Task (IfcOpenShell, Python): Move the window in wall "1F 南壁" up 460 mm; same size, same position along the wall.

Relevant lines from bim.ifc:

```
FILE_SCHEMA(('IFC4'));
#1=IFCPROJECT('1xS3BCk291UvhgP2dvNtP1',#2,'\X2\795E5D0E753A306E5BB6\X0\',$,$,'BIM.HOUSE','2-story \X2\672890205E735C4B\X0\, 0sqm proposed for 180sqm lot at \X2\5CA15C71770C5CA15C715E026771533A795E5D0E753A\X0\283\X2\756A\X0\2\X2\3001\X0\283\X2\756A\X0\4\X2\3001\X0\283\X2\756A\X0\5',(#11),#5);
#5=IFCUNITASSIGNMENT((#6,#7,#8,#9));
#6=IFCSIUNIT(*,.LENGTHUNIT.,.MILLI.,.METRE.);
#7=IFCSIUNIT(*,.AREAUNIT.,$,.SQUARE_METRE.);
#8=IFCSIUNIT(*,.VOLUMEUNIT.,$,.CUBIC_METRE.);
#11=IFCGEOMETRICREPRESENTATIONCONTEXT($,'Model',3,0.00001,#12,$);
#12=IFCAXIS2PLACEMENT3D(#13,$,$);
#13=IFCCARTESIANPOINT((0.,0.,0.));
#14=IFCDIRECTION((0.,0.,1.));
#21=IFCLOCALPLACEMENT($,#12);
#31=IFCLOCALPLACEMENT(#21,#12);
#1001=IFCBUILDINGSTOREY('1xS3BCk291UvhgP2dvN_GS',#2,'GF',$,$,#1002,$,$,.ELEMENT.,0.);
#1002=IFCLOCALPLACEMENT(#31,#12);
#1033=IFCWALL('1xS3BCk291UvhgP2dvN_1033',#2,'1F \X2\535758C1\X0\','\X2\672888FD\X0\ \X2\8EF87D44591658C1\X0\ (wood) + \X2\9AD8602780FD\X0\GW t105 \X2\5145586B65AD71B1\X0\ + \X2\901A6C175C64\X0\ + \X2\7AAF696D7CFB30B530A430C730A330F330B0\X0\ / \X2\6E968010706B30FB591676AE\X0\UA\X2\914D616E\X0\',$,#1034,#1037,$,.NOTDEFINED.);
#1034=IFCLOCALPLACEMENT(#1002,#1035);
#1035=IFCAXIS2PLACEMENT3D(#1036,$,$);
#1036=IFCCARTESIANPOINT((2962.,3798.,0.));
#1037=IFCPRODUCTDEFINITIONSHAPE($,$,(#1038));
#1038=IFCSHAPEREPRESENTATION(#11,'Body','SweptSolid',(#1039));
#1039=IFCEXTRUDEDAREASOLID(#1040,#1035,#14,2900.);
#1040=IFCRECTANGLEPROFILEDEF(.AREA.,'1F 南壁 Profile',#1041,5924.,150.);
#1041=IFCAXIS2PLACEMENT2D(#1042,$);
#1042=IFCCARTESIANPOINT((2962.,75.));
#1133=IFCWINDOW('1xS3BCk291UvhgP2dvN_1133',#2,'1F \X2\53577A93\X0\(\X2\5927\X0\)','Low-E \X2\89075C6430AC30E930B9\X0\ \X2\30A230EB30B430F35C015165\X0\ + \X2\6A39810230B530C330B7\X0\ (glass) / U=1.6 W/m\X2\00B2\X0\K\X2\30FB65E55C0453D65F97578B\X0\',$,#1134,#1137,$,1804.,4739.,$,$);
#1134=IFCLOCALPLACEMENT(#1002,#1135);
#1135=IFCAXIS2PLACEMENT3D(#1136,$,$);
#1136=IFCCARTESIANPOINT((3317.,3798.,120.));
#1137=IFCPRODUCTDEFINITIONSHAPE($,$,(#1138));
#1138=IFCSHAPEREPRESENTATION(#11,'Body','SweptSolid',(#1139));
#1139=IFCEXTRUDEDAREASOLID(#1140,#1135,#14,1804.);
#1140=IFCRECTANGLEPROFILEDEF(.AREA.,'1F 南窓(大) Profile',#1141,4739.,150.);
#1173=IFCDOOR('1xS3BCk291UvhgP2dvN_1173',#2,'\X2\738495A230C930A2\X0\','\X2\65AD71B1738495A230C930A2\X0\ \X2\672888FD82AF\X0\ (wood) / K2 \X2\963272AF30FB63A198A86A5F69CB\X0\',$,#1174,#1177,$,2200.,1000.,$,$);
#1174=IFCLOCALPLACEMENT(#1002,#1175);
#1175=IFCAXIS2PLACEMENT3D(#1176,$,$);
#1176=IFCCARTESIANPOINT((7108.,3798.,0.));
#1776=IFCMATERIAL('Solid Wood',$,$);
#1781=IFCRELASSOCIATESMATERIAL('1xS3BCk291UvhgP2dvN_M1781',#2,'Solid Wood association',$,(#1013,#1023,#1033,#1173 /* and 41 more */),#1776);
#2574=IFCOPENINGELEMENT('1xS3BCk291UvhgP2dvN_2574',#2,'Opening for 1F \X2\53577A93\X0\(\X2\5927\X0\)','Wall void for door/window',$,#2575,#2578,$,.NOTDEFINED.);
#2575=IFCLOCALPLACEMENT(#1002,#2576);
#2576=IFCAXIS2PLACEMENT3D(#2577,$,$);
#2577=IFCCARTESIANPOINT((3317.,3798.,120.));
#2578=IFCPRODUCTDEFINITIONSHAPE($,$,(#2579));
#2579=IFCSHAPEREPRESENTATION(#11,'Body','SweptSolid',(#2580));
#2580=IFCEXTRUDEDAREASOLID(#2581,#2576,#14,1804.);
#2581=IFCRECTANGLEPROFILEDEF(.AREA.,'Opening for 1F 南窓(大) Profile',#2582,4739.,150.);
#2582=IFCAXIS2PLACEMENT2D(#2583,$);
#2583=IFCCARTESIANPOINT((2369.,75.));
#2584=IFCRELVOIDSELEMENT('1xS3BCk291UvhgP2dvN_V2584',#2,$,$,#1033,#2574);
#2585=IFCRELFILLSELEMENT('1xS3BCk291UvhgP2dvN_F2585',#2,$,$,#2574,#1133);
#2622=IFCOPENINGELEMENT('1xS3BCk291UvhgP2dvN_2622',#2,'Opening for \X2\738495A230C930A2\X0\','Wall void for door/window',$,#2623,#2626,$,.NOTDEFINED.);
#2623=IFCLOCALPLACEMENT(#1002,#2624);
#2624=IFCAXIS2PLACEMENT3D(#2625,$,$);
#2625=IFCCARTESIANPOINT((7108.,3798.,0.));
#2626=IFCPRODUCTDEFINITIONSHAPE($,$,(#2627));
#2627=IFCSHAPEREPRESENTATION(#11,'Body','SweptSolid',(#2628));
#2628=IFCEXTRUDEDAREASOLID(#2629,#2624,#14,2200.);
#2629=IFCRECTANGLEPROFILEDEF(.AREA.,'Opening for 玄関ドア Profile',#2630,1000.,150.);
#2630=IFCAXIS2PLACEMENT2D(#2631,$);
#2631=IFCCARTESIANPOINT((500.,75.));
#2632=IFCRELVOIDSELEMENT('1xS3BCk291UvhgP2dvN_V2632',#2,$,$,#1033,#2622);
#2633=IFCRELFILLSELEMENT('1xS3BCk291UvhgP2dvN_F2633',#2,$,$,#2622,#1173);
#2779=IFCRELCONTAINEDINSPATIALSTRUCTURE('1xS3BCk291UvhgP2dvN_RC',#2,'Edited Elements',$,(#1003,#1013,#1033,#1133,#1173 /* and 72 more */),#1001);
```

```python
import numpy as np
import ifcopenshell
import ifcopenshell.api.geometry
import ifcopenshell.util.placement
import ifcopenshell.util.unit

model = ifcopenshell.open("bim.ifc")
unit_scale = ifcopenshell.util.unit.calculate_unit_scale(model)

window = model.by_guid("1xS3BCk291UvhgP2dvN_1133")
opening = window.FillsVoids[0].RelatingOpeningElement
dz = 460.0

shift = np.array([0.0, 0.0, dz])
# The window is not placed relative to its opening, so move both.
for product in (opening, window):
    matrix = ifcopenshell.util.placement.get_local_placement(product.ObjectPlacement)
    matrix[:3, 3] += shift
    ifcopenshell.api.geometry.edit_object_placement(model, product=product, matrix=matrix, is_si=False)

print(f"moved by {dz * unit_scale:+.3f} m")

model.write("bim-out.ifc")
```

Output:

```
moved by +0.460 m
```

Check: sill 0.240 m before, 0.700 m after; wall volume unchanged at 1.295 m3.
